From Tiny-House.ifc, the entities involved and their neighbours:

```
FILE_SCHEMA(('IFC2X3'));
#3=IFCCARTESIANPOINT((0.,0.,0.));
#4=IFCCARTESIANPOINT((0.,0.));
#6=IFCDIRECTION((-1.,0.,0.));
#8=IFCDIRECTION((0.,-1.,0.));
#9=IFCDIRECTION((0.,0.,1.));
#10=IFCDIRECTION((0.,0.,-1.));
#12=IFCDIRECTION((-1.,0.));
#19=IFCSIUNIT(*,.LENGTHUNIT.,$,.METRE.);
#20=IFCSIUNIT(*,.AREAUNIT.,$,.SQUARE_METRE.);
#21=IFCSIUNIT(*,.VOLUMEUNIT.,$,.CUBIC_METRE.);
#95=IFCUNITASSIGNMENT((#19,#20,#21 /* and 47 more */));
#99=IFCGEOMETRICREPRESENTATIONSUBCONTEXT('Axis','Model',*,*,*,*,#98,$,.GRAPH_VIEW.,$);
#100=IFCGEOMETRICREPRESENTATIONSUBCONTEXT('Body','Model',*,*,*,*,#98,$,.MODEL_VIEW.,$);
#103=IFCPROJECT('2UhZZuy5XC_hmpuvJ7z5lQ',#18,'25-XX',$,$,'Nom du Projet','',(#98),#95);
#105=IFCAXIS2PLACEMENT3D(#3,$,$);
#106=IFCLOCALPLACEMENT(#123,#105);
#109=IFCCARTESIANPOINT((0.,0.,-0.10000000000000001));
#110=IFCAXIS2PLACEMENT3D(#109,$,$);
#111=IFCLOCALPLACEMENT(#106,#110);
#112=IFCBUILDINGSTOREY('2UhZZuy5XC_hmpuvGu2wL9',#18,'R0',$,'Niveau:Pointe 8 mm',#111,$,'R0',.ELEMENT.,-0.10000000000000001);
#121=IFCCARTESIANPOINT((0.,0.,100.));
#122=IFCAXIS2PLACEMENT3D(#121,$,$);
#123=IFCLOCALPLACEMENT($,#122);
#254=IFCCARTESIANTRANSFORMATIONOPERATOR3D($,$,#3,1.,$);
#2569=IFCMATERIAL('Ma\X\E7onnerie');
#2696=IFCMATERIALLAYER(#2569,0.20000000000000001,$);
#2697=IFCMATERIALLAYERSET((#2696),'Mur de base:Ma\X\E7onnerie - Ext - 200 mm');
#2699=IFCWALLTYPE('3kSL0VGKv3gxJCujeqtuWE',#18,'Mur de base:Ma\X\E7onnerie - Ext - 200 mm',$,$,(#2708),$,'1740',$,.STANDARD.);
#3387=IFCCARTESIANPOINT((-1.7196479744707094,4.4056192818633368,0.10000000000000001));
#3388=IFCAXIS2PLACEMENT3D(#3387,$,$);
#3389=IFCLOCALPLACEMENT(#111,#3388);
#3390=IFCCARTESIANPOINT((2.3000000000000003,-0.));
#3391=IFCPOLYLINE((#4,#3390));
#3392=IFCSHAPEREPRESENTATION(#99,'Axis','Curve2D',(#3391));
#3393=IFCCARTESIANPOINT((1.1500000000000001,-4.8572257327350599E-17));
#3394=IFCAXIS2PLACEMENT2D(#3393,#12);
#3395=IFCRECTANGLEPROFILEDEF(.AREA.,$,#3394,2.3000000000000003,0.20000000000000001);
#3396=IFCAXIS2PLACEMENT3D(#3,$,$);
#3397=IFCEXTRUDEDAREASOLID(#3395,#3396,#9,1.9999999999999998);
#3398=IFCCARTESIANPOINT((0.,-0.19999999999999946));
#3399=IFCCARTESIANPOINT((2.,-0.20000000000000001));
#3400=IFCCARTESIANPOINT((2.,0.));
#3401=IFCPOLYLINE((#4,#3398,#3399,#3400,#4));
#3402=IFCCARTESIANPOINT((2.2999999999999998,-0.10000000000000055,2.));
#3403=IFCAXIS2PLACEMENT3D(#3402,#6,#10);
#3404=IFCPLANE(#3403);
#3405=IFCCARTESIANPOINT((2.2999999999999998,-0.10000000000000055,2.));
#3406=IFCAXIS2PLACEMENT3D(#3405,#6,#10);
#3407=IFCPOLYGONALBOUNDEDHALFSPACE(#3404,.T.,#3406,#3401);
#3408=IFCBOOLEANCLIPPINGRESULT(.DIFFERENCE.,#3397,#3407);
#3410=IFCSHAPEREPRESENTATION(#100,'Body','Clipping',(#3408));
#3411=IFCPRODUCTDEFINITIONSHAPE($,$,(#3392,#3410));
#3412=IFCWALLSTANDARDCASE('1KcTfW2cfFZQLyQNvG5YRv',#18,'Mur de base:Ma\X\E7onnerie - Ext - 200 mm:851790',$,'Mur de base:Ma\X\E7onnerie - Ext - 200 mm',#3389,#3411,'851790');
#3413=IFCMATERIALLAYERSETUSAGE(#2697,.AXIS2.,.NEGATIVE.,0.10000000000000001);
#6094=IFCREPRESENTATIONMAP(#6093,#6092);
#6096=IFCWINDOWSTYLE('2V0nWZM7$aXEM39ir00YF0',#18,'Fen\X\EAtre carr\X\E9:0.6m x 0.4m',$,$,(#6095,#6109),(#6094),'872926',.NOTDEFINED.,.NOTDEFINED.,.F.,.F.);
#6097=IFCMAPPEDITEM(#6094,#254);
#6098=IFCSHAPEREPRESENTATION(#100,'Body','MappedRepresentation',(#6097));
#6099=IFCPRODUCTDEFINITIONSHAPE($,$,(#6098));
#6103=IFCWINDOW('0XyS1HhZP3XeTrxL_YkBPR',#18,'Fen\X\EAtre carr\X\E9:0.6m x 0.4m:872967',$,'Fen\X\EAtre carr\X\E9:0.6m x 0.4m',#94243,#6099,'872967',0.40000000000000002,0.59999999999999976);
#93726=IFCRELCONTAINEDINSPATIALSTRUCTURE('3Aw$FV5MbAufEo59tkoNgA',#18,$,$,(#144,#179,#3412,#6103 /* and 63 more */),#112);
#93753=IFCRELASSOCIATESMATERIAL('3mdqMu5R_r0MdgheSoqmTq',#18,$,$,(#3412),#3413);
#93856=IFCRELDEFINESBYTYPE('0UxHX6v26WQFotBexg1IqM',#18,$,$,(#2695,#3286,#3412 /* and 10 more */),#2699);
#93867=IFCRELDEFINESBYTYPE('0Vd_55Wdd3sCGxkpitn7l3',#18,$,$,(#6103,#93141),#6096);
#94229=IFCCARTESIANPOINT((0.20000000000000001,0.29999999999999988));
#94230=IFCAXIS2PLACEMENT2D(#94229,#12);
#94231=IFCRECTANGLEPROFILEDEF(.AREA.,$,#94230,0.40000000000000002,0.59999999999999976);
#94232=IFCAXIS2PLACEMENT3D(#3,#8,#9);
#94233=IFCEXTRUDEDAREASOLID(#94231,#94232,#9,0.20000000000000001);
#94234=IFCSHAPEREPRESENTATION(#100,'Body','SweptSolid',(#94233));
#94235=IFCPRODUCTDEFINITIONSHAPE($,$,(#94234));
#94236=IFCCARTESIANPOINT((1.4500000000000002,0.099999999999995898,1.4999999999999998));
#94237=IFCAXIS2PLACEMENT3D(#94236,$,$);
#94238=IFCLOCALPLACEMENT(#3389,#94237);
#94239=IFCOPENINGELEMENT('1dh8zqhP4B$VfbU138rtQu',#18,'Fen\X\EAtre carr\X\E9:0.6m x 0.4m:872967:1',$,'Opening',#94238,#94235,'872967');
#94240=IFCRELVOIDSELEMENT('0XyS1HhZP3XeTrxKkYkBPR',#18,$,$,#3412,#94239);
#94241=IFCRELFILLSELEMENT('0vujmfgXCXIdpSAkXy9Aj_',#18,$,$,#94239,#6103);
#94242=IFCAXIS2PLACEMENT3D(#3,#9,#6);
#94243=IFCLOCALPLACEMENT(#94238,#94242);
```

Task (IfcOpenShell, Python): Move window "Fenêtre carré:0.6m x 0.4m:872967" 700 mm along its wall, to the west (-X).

```python
import ifcopenshell
import ifcopenshell.api.geometry
import ifcopenshell.util.placement
import ifcopenshell.util.unit

model = ifcopenshell.open("Tiny-House.ifc")
unit_scale = ifcopenshell.util.unit.calculate_unit_scale(model)

window = model.by_guid("0XyS1HhZP3XeTrxL_YkBPR")
opening = window.FillsVoids[0].RelatingOpeningElement
wall = opening.VoidsElements[0].RelatingBuildingElement

wall_matrix = ifcopenshell.util.placement.get_local_placement(wall.ObjectPlacement)
shift = wall_matrix[:3, 0] * -0.7 / unit_scale
before = ifcopenshell.util.placement.get_local_placement(window.ObjectPlacement)[:3, 3].copy()

# The window is placed relative to its opening, so it follows when the opening moves.
matrix = ifcopenshell.util.placement.get_local_placement(opening.ObjectPlacement)
matrix[:3, 3] += shift
ifcopenshell.api.geometry.edit_object_placement(
    model, product=opening, matrix=matrix, is_si=False, should_transform_children=True
)

after = ifcopenshell.util.placement.get_local_placement(window.ObjectPlacement)[:3, 3]
print("window moved by", (after - before).round(3) + 0.0)

model.write("Tiny-House-out.ifc")
```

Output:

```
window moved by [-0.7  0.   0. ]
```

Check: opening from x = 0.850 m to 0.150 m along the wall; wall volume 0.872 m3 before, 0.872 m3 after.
